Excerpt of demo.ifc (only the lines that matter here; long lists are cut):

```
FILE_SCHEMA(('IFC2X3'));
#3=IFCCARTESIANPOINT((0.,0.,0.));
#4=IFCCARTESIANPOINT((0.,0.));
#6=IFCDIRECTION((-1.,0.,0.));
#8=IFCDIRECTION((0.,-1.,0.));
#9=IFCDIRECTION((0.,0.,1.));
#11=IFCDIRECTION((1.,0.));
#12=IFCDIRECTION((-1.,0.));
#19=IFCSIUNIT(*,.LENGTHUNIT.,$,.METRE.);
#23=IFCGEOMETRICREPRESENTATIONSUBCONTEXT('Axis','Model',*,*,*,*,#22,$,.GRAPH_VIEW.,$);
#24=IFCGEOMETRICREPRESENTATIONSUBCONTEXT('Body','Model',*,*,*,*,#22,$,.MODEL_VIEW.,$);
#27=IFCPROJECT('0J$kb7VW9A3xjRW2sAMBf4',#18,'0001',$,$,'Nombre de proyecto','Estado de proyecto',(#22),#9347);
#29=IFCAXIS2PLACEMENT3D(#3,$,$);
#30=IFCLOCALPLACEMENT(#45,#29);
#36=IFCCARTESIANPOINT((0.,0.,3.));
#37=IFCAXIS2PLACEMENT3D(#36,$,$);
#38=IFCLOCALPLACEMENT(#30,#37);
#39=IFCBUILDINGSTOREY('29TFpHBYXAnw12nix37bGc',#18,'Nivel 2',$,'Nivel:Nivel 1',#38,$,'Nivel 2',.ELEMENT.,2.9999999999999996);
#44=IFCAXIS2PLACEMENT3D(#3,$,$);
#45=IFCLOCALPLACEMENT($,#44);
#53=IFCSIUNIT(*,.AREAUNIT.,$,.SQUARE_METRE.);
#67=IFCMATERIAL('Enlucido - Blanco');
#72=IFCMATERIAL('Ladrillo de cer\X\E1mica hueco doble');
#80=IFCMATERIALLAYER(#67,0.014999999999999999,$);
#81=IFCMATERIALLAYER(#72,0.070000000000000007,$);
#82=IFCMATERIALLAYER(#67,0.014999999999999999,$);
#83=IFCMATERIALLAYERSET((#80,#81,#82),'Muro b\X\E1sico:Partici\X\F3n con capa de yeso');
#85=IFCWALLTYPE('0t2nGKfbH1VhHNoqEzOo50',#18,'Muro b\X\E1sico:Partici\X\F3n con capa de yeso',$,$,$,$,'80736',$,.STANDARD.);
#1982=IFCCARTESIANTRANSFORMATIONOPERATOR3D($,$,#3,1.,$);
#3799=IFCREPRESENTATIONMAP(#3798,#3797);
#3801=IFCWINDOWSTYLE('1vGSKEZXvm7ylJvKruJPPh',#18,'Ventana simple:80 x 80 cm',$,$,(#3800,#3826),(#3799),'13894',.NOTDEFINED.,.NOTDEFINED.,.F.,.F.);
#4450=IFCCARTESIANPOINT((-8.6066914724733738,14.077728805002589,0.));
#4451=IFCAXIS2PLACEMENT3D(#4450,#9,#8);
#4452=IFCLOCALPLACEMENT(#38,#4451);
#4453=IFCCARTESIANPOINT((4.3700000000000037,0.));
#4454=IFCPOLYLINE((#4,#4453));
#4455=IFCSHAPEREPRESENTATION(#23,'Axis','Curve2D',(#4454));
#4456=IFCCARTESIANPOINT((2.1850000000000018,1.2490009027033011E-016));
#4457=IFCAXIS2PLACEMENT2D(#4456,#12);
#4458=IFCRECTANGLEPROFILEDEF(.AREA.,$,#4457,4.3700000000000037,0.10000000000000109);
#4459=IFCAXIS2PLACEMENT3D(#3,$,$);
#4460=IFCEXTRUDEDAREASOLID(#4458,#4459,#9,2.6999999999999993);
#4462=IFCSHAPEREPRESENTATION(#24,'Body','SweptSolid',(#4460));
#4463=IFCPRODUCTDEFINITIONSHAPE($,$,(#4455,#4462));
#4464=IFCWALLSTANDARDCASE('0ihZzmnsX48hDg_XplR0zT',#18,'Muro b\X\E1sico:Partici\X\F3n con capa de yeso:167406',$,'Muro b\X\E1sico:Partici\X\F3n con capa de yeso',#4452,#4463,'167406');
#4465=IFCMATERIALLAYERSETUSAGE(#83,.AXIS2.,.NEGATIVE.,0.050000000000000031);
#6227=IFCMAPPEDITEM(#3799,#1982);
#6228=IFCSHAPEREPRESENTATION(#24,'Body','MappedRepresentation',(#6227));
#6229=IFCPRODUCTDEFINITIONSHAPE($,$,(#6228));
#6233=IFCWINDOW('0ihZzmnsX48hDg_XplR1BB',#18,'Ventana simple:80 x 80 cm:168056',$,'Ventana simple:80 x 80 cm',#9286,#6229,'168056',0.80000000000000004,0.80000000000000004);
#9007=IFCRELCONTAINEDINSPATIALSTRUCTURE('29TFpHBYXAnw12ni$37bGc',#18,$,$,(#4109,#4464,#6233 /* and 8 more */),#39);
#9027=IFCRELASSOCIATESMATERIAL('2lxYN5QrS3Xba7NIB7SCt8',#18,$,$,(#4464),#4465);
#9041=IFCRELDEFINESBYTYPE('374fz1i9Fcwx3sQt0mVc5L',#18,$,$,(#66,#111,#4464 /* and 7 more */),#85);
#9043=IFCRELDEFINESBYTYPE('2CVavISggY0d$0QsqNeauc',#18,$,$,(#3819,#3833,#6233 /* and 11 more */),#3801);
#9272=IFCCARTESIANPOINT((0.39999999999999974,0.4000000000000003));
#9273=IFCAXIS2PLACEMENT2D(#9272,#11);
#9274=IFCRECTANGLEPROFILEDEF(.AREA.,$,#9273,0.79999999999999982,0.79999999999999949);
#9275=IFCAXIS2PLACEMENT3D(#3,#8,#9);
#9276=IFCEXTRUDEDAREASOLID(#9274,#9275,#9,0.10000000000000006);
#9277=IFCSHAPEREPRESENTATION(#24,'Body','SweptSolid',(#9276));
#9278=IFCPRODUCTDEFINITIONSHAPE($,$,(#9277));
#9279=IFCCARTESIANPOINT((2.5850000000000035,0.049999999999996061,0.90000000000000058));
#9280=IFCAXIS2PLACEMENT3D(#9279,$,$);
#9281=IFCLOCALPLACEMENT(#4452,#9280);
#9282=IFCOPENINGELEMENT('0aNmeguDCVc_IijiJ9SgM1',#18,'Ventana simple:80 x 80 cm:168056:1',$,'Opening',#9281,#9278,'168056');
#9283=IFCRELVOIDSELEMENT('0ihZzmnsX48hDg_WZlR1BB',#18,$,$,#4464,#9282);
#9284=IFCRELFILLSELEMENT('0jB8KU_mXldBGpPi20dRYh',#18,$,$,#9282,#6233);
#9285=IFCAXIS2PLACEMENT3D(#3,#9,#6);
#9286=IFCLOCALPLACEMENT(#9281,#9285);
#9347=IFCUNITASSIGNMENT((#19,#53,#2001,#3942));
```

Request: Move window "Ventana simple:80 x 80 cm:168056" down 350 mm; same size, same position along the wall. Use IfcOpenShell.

```python
import numpy as np
import ifcopenshell
import ifcopenshell.api.geometry
import ifcopenshell.util.placement
import ifcopenshell.util.unit

model = ifcopenshell.open("demo.ifc")
unit_scale = ifcopenshell.util.unit.calculate_unit_scale(model)

window = model.by_id(6233)
opening = window.FillsVoids[0].RelatingOpeningElement
dz = -0.35 / unit_scale

shift = np.array([0.0, 0.0, dz])
# The window is placed relative to its opening, so it follows when the opening moves.
matrix = ifcopenshell.util.placement.get_local_placement(opening.ObjectPlacement)
matrix[:3, 3] += shift
ifcopenshell.api.geometry.edit_object_placement(
    model, product=opening, matrix=matrix, is_si=False, should_transform_children=True
)

print(f"moved by {dz * unit_scale:+.3f} m")

model.write("demo-out.ifc")
```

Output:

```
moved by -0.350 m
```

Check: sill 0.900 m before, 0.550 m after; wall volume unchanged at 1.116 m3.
